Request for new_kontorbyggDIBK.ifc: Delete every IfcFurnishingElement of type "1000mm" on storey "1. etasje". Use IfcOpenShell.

First a look at what the model holds.

```python
import ifcopenshell
import ifcopenshell.util.element

model = ifcopenshell.open("new_kontorbyggDIBK.ifc")
print(model.schema)
storey = next(s for s in model.by_type("IfcBuildingStorey") if s.Name == "1. etasje")
furniture = [e for e in ifcopenshell.util.element.get_decomposition(storey) if e.is_a("IfcFurnishingElement")]
seen = {}
for e in furniture:
    element_type = ifcopenshell.util.element.get_type(e)
    name = element_type.Name if element_type not in (None, e) else None
    seen[name] = seen.get(name, 0) + 1
for name, count in sorted(seen.items(), key=str):
    print(count, "x", name)
```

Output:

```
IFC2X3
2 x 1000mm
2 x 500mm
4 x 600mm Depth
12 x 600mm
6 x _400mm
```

```python
import ifcopenshell
import ifcopenshell.api.root
import ifcopenshell.util.element

model = ifcopenshell.open("new_kontorbyggDIBK.ifc")

storey = next(s for s in model.by_type("IfcBuildingStorey") if s.Name == "1. etasje")
furniture = [e for e in ifcopenshell.util.element.get_decomposition(storey) if e.is_a("IfcFurnishingElement")]
targets = [e for e in furniture if (t := ifcopenshell.util.element.get_type(e)) not in (None, e) and t.Name == "1000mm"]

for e in targets:
    ifcopenshell.api.root.remove_product(model, product=e)
print(len(targets), "removed")

model.write("new_kontorbyggDIBK-out.ifc")
```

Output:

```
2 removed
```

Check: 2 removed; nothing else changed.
